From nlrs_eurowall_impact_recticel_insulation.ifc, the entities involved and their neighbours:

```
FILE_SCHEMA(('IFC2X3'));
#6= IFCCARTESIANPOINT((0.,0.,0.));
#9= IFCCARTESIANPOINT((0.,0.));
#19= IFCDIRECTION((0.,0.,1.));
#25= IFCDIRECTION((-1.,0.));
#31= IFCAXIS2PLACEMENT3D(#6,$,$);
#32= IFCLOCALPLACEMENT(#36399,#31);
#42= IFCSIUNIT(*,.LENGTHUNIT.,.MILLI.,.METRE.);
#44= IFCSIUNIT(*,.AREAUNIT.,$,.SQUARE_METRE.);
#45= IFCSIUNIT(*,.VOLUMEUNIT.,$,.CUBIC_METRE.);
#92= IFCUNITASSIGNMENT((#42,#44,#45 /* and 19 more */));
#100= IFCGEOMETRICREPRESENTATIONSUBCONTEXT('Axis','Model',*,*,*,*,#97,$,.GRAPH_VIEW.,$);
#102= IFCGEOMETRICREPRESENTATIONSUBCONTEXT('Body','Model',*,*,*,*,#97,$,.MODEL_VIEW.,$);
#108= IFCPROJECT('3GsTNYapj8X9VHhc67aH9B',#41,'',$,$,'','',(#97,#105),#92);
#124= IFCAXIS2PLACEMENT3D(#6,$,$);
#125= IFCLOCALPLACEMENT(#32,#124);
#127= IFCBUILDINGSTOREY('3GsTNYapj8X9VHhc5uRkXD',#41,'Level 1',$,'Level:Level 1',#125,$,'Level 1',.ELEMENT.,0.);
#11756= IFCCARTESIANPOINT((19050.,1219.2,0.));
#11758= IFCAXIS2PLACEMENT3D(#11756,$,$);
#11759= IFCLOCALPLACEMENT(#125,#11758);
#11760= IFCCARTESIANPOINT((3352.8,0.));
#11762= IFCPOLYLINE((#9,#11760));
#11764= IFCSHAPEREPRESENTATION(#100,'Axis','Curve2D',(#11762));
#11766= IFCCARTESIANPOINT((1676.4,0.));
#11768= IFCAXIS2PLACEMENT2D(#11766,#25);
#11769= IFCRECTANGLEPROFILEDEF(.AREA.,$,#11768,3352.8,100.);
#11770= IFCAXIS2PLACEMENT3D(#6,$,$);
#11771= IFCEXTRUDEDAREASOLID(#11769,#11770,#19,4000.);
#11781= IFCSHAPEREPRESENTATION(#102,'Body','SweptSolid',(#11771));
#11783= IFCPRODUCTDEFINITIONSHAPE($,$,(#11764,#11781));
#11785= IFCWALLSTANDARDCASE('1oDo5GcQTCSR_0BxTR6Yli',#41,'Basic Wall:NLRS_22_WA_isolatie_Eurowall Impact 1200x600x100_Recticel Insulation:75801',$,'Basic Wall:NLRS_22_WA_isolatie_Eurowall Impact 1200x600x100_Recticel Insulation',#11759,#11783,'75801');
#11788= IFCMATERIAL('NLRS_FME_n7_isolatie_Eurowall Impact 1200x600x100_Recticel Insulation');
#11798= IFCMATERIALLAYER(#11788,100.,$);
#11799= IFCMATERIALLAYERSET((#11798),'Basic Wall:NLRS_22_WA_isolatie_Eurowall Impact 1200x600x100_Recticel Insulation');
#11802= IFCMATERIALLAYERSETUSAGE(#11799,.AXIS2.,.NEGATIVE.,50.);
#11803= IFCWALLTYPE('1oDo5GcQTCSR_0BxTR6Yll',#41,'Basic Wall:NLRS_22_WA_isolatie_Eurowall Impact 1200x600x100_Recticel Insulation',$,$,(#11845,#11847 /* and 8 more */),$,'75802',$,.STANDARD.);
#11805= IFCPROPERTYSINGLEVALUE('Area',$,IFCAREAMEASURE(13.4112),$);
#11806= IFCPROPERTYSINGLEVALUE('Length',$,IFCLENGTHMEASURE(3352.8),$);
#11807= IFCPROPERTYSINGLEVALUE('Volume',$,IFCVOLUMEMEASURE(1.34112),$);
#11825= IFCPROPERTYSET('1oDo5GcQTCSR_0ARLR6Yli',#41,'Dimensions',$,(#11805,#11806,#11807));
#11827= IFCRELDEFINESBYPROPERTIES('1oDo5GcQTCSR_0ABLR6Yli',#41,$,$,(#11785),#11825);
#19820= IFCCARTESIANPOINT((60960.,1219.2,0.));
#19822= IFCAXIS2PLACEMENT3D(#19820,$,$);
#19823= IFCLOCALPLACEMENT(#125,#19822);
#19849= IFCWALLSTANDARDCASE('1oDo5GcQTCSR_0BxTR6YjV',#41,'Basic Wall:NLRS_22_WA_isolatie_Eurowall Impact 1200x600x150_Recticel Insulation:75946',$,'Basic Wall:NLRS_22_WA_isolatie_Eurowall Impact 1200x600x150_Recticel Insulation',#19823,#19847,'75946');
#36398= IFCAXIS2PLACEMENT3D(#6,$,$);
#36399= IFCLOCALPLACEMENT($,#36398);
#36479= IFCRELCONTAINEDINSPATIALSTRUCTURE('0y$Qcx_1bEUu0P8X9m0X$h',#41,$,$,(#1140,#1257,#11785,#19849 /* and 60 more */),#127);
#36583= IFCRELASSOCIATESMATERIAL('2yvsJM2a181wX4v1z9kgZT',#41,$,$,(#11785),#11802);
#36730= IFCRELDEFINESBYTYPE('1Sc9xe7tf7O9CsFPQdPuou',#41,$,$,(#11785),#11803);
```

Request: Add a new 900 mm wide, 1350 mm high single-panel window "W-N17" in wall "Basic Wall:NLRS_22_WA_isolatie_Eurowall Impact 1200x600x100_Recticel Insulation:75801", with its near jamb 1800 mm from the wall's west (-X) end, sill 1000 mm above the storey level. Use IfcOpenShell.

```python
import numpy as np
import ifcopenshell
import ifcopenshell.api.feature
import ifcopenshell.api.geometry
import ifcopenshell.api.pset
import ifcopenshell.api.root
import ifcopenshell.api.spatial
import ifcopenshell.api.type
import ifcopenshell.geom
import ifcopenshell.util.element
import ifcopenshell.util.placement
import ifcopenshell.util.representation
import ifcopenshell.util.shape
import ifcopenshell.util.unit

model = ifcopenshell.open("nlrs_eurowall_impact_recticel_insulation.ifc")
unit_scale = ifcopenshell.util.unit.calculate_unit_scale(model)
area_scale = ifcopenshell.util.unit.calculate_unit_scale(model, "AREAUNIT")
volume_scale = ifcopenshell.util.unit.calculate_unit_scale(model, "VOLUMEUNIT")
settings = ifcopenshell.geom.settings()


def volume(element):
    """Net volume in cubic metres, openings subtracted."""
    shape = ifcopenshell.geom.create_shape(settings, element)
    return ifcopenshell.util.shape.get_volume(shape.geometry)


wall = model.by_guid("1oDo5GcQTCSR_0BxTR6Yli")
storey = ifcopenshell.util.element.get_container(wall, ifc_class="IfcBuildingStorey")
context = ifcopenshell.util.representation.get_context(model, "Model", "Body", "MODEL_VIEW")
before = volume(wall)

width, height, from_end, sill = 0.9, 1.35, 1.8, 1  # metres

# The wall runs along its own X axis, and the end named is its -X end.
wall_shape = ifcopenshell.geom.create_shape(settings, wall)
x, y, z = ifcopenshell.util.shape.get_vertices(wall_shape.geometry).T
start = x.min() + from_end
face, thickness = float(y.min()), float(y.max() - y.min())
wall_matrix = ifcopenshell.util.placement.get_local_placement(wall.ObjectPlacement)
level = ifcopenshell.util.placement.get_local_placement(storey.ObjectPlacement)[2, 3]


def in_wall(x, y):
    """Placement at x, y metres in the wall's axes, at sill height."""
    matrix = wall_matrix.copy()
    matrix[:, 3] = wall_matrix @ np.array([x / unit_scale, y / unit_scale, 0.0, 1.0])
    matrix[2, 3] = level + sill / unit_scale
    return matrix


# Opening: a box that overshoots both wall faces by 50 mm.
opening = ifcopenshell.api.root.create_entity(model, ifc_class="IfcOpeningElement")
box = ifcopenshell.api.geometry.add_wall_representation(
    model, context=context, length=width, height=height, thickness=thickness + 0.1
)
ifcopenshell.api.geometry.assign_representation(model, product=opening, representation=box)
ifcopenshell.api.geometry.edit_object_placement(model, product=opening, matrix=in_wall(start, face - 0.05), is_si=False)
ifcopenshell.api.feature.add_feature(model, feature=opening, element=wall)

window = ifcopenshell.api.root.create_entity(model, ifc_class="IfcWindow", name="W-N17")
window.OverallWidth, window.OverallHeight = width / unit_scale, height / unit_scale
body = ifcopenshell.api.geometry.add_window_representation(
    model,
    context=context,
    overall_width=window.OverallWidth,
    overall_height=window.OverallHeight,
    partition_type="SINGLE_PANEL",
)
ifcopenshell.api.geometry.assign_representation(model, product=window, representation=body)
ifcopenshell.api.spatial.assign_container(model, products=[window], relating_structure=storey)
fills = ifcopenshell.api.feature.add_filling(model, opening=opening, element=window)
fills.OwnerHistory = window.OwnerHistory  # required in IFC2X3

# IFC2X3 keeps the operation on the window style.
style = ifcopenshell.api.root.create_entity(model, ifc_class="IfcWindowStyle", name="W-N17")
style.OperationType, style.ConstructionType = "SINGLE_PANEL", "NOTDEFINED"
style.ParameterTakesPrecedence = style.Sizeable = False
ifcopenshell.api.type.assign_type(model, related_objects=[window], relating_type=style)

# Centre the window in the wall's thickness.
ifcopenshell.api.geometry.edit_object_placement(model, product=window, matrix=in_wall(start, face), is_si=False)
window_shape = ifcopenshell.geom.create_shape(settings, window)
depth = ifcopenshell.util.shape.get_vertices(window_shape.geometry)[:, 1]
offset = face + thickness / 2 - (depth.min() + depth.max()) / 2
ifcopenshell.api.geometry.edit_object_placement(model, product=window, matrix=in_wall(start, offset), is_si=False)

after = volume(wall)

# Update the wall's stored quantities.
pset = model.by_id(ifcopenshell.util.element.get_pset(wall, "Dimensions", should_inherit=False)["id"])
ifcopenshell.api.pset.edit_pset(model, pset=pset, properties={
    "Area": model.create_entity("IfcAreaMeasure", after / thickness / area_scale),
    "Volume": model.create_entity("IfcVolumeMeasure", after / volume_scale),
})

print(f"wall volume {before:.3f} -> {after:.3f} m3")

model.write("nlrs_eurowall_impact_recticel_insulation_updated.ifc")
```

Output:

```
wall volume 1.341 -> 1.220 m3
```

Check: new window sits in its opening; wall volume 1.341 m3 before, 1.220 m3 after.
